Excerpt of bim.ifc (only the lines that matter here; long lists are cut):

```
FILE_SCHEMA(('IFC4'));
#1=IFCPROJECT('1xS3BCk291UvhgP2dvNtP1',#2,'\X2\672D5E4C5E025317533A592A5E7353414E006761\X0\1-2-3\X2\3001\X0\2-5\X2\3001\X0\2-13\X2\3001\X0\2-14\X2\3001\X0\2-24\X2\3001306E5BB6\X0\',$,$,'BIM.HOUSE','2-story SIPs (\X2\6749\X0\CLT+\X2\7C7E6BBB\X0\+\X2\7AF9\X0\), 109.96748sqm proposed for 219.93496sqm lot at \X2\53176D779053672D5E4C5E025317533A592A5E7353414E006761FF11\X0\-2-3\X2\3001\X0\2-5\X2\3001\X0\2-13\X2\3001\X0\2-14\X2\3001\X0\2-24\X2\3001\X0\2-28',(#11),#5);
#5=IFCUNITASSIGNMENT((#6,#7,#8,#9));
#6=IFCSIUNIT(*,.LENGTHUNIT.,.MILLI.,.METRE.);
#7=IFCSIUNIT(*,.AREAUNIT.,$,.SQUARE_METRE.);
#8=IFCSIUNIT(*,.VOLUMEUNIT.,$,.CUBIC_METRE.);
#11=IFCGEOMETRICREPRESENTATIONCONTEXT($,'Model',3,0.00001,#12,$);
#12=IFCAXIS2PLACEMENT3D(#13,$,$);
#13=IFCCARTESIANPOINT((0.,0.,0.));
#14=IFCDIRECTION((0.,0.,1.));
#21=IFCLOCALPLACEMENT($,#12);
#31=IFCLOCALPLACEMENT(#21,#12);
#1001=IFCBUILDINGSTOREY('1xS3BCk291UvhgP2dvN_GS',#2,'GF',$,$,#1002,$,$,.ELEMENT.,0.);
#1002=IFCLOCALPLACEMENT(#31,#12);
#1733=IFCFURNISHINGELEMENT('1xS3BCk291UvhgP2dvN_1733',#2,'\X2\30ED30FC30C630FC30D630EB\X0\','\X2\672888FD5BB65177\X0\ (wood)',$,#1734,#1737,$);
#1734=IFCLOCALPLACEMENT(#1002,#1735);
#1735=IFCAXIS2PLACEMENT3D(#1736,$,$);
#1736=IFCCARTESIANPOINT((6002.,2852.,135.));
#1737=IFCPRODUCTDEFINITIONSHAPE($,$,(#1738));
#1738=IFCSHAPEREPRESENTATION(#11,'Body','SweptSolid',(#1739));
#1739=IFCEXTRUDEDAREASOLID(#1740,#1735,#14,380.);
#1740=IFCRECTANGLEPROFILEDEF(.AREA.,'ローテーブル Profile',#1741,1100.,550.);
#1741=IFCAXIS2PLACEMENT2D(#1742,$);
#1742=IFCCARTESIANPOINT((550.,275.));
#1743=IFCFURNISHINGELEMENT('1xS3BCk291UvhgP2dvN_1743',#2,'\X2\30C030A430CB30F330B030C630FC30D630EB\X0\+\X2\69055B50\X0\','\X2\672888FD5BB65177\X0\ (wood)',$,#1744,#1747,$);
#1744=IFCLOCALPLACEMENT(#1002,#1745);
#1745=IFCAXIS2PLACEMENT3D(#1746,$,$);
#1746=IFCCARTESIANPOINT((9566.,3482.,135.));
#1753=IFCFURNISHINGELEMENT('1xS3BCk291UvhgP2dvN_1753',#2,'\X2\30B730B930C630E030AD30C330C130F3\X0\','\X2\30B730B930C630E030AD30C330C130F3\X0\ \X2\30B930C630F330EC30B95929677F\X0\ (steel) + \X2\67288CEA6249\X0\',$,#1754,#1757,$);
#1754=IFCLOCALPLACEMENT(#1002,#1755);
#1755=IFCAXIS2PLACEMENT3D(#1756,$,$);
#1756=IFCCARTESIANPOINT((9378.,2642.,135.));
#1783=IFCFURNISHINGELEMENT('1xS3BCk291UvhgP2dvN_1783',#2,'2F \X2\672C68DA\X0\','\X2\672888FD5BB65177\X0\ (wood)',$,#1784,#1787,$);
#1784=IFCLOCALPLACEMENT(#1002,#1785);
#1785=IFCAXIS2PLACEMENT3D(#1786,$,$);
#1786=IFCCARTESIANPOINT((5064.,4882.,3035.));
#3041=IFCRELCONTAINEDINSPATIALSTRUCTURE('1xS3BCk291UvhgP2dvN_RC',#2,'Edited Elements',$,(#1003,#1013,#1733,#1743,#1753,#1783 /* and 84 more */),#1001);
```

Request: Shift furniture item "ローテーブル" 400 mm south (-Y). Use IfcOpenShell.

```python
import ifcopenshell
import ifcopenshell.api.geometry
import ifcopenshell.util.placement

model = ifcopenshell.open("bim.ifc")

item = model.by_id(1733)
matrix = ifcopenshell.util.placement.get_local_placement(item.ObjectPlacement)
matrix[1, 3] -= 400.0
ifcopenshell.api.geometry.edit_object_placement(model, product=item, matrix=matrix, is_si=False)

print(ifcopenshell.util.placement.get_local_placement(item.ObjectPlacement).round(3) + 0.0)

model.write("bim_v2.ifc")
```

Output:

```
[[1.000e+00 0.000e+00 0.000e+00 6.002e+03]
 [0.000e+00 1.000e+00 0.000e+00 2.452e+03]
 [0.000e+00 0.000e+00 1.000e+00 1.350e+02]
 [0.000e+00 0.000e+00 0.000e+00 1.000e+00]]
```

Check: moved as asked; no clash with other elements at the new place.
